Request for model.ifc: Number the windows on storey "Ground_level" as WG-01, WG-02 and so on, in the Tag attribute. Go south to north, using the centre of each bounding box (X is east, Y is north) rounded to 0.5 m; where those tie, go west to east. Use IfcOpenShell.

First a look at what the model holds.

```python
import ifcopenshell
import ifcopenshell.util.element
import ifcopenshell.util.placement

model = ifcopenshell.open("model.ifc")
print(model.schema)
storey = next(s for s in model.by_type("IfcBuildingStorey") if s.Name == "Ground_level")
windows = [e for e in ifcopenshell.util.element.get_decomposition(storey) if e.is_a("IfcWindow")]
for e in sorted(windows, key=lambda e: e.id()):
    origin = ifcopenshell.util.placement.get_local_placement(e.ObjectPlacement)[:3, 3]
    print(e.id(), e.Tag, e.Name, origin.round(2) + 0.0, sep=" | ")
```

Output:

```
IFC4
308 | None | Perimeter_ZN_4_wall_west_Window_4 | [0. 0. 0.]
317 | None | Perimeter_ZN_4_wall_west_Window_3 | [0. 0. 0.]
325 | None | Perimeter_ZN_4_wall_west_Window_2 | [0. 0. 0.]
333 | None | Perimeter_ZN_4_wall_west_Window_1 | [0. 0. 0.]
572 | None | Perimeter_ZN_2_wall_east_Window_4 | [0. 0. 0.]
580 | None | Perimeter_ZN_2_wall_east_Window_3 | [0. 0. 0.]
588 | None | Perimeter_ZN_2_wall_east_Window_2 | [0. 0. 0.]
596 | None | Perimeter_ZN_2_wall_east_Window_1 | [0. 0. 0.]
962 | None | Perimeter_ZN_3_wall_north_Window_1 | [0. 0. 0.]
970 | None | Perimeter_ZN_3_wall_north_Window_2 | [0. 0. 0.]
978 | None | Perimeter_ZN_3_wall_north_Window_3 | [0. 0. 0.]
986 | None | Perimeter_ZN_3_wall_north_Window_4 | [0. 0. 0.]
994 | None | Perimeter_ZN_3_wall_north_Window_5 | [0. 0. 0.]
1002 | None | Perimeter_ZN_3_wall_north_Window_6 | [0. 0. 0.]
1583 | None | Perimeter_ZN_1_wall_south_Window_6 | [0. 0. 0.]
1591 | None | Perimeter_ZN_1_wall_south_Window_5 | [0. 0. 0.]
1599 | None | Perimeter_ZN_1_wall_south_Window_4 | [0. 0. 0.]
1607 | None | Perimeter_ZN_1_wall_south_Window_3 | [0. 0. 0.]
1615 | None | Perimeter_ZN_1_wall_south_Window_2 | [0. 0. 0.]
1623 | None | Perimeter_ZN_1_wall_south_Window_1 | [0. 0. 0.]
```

```python
import ifcopenshell
import ifcopenshell.geom
import ifcopenshell.util.element
import ifcopenshell.util.shape

model = ifcopenshell.open("model.ifc")
settings = ifcopenshell.geom.settings()
settings.set("use-world-coords", True)


def centre(element):
    shape = ifcopenshell.geom.create_shape(settings, element)
    return ifcopenshell.util.shape.get_bbox_centroid(shape.geometry)


storey = next(s for s in model.by_type("IfcBuildingStorey") if s.Name == "Ground_level")
windows = [e for e in ifcopenshell.util.element.get_decomposition(storey) if e.is_a("IfcWindow")]

# Insertion points can sit at a corner or the storey origin, so sort by the geometry (in metres).
centres = {e: centre(e) for e in windows}
windows.sort(key=lambda e: (round(centres[e][1] / 0.5), centres[e][0]))

for i, e in enumerate(windows, start=1):
    number = f"WG-{i:02d}"
    e.Tag = number
    print(e.id(), number)

model.write("model_rev.ifc")
```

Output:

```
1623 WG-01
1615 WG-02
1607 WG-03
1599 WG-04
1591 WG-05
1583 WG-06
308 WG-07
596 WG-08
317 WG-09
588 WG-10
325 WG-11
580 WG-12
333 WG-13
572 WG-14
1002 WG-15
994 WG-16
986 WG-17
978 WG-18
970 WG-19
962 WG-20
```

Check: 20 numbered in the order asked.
